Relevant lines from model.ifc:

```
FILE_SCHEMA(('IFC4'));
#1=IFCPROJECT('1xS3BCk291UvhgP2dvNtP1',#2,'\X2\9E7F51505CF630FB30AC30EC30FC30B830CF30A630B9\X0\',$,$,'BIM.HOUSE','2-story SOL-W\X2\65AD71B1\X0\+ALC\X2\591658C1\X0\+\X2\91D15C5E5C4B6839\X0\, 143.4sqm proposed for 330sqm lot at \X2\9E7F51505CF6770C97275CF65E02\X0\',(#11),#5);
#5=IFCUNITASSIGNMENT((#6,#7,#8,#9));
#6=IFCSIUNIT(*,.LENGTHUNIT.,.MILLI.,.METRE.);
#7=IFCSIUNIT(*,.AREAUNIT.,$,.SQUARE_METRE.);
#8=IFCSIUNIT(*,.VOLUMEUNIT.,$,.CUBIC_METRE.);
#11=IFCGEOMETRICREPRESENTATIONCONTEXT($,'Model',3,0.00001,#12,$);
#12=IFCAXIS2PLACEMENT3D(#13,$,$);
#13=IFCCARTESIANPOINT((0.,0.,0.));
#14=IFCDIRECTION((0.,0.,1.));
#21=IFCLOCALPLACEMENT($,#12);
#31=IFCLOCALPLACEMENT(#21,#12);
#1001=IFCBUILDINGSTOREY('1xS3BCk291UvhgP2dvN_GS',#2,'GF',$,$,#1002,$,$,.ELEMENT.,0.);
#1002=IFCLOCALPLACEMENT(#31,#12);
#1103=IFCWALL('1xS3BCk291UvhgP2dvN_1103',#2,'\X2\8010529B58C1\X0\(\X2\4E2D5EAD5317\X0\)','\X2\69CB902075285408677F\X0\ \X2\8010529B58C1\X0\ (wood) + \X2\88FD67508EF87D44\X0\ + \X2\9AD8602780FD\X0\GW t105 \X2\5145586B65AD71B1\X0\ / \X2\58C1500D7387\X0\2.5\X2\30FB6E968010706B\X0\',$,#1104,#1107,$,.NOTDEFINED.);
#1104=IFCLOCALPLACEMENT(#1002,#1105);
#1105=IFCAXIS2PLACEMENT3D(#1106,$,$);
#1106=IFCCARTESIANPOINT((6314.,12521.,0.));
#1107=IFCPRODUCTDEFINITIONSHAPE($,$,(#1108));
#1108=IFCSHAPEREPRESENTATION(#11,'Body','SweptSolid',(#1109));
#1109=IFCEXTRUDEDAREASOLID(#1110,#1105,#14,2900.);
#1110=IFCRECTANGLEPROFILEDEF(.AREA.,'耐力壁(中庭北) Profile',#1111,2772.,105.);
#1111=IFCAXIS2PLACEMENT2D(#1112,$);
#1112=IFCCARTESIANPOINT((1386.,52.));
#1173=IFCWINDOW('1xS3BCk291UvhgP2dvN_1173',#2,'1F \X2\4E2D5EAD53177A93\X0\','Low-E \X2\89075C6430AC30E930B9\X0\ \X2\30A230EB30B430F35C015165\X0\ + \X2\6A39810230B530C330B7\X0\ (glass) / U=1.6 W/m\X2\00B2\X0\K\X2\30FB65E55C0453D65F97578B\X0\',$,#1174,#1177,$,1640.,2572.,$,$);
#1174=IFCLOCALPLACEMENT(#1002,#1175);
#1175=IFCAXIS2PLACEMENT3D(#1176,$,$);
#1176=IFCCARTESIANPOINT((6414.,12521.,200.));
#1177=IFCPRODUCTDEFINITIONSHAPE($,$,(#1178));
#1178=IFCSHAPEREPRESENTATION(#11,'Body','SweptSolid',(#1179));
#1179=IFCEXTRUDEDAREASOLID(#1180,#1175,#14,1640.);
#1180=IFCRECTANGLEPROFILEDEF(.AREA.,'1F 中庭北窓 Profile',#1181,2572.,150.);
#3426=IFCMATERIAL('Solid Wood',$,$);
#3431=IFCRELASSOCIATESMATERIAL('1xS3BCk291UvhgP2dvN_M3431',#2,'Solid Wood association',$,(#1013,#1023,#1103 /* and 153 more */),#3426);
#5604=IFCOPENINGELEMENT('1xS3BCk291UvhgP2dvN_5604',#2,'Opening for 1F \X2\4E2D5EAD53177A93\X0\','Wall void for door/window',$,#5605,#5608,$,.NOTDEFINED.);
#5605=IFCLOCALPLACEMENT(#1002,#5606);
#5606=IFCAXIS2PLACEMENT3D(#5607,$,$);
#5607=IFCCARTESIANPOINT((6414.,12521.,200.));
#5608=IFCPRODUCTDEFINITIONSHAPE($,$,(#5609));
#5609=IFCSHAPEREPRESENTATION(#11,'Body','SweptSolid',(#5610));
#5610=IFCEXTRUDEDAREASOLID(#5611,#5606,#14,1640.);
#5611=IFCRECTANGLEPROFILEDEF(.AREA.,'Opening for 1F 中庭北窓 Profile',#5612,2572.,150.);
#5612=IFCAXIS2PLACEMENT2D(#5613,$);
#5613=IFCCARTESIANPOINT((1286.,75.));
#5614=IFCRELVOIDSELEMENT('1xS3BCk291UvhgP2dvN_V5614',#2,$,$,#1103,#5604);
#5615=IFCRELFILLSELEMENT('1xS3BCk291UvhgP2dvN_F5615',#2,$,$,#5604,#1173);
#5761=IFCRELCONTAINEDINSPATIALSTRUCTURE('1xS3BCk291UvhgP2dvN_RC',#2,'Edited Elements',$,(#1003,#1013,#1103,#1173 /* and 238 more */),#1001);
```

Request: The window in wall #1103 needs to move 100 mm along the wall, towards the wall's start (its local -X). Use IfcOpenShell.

```python
import ifcopenshell
import ifcopenshell.api.geometry
import ifcopenshell.util.placement

model = ifcopenshell.open("model.ifc")

window = model.by_guid("1xS3BCk291UvhgP2dvN_1173")
opening = window.FillsVoids[0].RelatingOpeningElement
wall = opening.VoidsElements[0].RelatingBuildingElement

wall_matrix = ifcopenshell.util.placement.get_local_placement(wall.ObjectPlacement)
shift = wall_matrix[:3, 0] * -100.0
before = ifcopenshell.util.placement.get_local_placement(window.ObjectPlacement)[:3, 3].copy()

# The window is not placed relative to its opening, so move both.
for product in (opening, window):
    matrix = ifcopenshell.util.placement.get_local_placement(product.ObjectPlacement)
    matrix[:3, 3] += shift
    ifcopenshell.api.geometry.edit_object_placement(model, product=product, matrix=matrix, is_si=False)

after = ifcopenshell.util.placement.get_local_placement(window.ObjectPlacement)[:3, 3]
print("window moved by", (after - before).round(3) + 0.0)

model.write("model_rev.ifc")
```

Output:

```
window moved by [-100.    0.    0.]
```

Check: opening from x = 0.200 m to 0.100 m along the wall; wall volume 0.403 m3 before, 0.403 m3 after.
